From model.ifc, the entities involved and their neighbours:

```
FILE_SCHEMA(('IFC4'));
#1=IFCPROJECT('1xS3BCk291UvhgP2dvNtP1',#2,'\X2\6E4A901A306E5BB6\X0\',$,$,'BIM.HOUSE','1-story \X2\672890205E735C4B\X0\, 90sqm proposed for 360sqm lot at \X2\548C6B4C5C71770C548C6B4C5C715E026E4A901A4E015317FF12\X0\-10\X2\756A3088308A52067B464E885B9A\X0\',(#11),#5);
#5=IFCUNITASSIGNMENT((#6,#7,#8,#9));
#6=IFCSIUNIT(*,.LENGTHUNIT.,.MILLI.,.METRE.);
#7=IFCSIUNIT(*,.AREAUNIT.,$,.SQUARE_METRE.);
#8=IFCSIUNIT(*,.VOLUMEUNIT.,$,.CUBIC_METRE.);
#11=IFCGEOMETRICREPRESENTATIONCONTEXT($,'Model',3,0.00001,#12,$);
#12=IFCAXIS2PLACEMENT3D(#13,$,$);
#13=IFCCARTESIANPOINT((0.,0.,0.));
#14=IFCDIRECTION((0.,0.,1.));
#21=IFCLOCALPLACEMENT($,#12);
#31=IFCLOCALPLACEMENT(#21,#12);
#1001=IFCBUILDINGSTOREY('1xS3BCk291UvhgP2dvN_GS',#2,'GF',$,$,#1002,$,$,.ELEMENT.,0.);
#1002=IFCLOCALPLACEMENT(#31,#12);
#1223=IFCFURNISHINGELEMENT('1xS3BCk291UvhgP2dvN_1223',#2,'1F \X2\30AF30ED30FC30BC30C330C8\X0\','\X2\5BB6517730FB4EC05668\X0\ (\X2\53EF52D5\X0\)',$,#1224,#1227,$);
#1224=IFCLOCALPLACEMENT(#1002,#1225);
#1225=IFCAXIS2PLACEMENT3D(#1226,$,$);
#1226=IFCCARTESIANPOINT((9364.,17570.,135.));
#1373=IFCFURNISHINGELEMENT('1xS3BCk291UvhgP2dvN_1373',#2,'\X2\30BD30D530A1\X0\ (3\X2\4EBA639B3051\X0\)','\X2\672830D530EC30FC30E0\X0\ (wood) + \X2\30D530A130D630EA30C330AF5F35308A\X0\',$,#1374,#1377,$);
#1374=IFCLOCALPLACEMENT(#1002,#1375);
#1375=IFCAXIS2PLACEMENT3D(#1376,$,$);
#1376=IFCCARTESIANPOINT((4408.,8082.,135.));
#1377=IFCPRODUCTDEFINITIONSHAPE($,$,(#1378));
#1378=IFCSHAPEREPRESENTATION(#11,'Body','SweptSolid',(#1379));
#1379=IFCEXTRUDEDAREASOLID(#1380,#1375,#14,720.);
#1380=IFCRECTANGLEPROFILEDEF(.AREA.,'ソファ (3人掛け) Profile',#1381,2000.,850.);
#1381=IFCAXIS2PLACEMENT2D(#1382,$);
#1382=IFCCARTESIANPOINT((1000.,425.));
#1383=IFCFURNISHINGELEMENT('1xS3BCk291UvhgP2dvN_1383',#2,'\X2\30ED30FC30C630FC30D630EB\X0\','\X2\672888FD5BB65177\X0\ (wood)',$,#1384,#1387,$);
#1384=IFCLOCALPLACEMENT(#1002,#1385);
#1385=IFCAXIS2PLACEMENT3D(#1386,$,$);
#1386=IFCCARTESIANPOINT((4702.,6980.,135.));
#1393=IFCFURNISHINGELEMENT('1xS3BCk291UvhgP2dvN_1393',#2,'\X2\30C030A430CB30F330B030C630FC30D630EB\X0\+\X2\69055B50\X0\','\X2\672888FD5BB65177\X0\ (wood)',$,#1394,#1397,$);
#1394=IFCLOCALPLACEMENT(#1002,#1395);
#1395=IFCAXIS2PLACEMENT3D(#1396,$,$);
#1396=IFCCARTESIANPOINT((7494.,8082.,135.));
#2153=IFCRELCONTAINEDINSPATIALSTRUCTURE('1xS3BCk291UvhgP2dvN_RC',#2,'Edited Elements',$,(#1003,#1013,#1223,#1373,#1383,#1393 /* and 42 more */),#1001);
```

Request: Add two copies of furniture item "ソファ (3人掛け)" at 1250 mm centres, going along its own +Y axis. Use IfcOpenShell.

```python
import ifcopenshell
import ifcopenshell.api.geometry
import ifcopenshell.api.root
import ifcopenshell.util.element
import ifcopenshell.util.placement

model = ifcopenshell.open("model.ifc")


def reuse_history(source, copy):
    """copy_class also copies each property set's owner history, people and application; keep the originals."""
    for rel in copy.IsDefinedBy:
        if rel.is_a("IfcRelDefinesByProperties") and (history := rel.RelatingPropertyDefinition.OwnerHistory):
            rel.RelatingPropertyDefinition.OwnerHistory = source.OwnerHistory
            ifcopenshell.util.element.remove_deep2(model, history)


source = model.by_id(1373)
base = ifcopenshell.util.placement.get_local_placement(source.ObjectPlacement)
step = base[:3, 1] * 1250.0

for i in range(1, 3):
    copy = ifcopenshell.api.root.copy_class(model, product=source)
    copy.Representation = ifcopenshell.util.element.copy_deep(
        model, source.Representation, exclude=["IfcGeometricRepresentationContext", "IfcRepresentationMap"]
    )
    reuse_history(source, copy)
    matrix = base.copy()
    matrix[:3, 3] += i * step
    print("added at", matrix[:3, 3].round(3) + 0.0)
    ifcopenshell.api.geometry.edit_object_placement(model, product=copy, matrix=matrix, is_si=False)

model.write("model_updated.ifc")
```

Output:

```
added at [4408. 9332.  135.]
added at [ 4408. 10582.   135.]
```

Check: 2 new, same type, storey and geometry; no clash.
